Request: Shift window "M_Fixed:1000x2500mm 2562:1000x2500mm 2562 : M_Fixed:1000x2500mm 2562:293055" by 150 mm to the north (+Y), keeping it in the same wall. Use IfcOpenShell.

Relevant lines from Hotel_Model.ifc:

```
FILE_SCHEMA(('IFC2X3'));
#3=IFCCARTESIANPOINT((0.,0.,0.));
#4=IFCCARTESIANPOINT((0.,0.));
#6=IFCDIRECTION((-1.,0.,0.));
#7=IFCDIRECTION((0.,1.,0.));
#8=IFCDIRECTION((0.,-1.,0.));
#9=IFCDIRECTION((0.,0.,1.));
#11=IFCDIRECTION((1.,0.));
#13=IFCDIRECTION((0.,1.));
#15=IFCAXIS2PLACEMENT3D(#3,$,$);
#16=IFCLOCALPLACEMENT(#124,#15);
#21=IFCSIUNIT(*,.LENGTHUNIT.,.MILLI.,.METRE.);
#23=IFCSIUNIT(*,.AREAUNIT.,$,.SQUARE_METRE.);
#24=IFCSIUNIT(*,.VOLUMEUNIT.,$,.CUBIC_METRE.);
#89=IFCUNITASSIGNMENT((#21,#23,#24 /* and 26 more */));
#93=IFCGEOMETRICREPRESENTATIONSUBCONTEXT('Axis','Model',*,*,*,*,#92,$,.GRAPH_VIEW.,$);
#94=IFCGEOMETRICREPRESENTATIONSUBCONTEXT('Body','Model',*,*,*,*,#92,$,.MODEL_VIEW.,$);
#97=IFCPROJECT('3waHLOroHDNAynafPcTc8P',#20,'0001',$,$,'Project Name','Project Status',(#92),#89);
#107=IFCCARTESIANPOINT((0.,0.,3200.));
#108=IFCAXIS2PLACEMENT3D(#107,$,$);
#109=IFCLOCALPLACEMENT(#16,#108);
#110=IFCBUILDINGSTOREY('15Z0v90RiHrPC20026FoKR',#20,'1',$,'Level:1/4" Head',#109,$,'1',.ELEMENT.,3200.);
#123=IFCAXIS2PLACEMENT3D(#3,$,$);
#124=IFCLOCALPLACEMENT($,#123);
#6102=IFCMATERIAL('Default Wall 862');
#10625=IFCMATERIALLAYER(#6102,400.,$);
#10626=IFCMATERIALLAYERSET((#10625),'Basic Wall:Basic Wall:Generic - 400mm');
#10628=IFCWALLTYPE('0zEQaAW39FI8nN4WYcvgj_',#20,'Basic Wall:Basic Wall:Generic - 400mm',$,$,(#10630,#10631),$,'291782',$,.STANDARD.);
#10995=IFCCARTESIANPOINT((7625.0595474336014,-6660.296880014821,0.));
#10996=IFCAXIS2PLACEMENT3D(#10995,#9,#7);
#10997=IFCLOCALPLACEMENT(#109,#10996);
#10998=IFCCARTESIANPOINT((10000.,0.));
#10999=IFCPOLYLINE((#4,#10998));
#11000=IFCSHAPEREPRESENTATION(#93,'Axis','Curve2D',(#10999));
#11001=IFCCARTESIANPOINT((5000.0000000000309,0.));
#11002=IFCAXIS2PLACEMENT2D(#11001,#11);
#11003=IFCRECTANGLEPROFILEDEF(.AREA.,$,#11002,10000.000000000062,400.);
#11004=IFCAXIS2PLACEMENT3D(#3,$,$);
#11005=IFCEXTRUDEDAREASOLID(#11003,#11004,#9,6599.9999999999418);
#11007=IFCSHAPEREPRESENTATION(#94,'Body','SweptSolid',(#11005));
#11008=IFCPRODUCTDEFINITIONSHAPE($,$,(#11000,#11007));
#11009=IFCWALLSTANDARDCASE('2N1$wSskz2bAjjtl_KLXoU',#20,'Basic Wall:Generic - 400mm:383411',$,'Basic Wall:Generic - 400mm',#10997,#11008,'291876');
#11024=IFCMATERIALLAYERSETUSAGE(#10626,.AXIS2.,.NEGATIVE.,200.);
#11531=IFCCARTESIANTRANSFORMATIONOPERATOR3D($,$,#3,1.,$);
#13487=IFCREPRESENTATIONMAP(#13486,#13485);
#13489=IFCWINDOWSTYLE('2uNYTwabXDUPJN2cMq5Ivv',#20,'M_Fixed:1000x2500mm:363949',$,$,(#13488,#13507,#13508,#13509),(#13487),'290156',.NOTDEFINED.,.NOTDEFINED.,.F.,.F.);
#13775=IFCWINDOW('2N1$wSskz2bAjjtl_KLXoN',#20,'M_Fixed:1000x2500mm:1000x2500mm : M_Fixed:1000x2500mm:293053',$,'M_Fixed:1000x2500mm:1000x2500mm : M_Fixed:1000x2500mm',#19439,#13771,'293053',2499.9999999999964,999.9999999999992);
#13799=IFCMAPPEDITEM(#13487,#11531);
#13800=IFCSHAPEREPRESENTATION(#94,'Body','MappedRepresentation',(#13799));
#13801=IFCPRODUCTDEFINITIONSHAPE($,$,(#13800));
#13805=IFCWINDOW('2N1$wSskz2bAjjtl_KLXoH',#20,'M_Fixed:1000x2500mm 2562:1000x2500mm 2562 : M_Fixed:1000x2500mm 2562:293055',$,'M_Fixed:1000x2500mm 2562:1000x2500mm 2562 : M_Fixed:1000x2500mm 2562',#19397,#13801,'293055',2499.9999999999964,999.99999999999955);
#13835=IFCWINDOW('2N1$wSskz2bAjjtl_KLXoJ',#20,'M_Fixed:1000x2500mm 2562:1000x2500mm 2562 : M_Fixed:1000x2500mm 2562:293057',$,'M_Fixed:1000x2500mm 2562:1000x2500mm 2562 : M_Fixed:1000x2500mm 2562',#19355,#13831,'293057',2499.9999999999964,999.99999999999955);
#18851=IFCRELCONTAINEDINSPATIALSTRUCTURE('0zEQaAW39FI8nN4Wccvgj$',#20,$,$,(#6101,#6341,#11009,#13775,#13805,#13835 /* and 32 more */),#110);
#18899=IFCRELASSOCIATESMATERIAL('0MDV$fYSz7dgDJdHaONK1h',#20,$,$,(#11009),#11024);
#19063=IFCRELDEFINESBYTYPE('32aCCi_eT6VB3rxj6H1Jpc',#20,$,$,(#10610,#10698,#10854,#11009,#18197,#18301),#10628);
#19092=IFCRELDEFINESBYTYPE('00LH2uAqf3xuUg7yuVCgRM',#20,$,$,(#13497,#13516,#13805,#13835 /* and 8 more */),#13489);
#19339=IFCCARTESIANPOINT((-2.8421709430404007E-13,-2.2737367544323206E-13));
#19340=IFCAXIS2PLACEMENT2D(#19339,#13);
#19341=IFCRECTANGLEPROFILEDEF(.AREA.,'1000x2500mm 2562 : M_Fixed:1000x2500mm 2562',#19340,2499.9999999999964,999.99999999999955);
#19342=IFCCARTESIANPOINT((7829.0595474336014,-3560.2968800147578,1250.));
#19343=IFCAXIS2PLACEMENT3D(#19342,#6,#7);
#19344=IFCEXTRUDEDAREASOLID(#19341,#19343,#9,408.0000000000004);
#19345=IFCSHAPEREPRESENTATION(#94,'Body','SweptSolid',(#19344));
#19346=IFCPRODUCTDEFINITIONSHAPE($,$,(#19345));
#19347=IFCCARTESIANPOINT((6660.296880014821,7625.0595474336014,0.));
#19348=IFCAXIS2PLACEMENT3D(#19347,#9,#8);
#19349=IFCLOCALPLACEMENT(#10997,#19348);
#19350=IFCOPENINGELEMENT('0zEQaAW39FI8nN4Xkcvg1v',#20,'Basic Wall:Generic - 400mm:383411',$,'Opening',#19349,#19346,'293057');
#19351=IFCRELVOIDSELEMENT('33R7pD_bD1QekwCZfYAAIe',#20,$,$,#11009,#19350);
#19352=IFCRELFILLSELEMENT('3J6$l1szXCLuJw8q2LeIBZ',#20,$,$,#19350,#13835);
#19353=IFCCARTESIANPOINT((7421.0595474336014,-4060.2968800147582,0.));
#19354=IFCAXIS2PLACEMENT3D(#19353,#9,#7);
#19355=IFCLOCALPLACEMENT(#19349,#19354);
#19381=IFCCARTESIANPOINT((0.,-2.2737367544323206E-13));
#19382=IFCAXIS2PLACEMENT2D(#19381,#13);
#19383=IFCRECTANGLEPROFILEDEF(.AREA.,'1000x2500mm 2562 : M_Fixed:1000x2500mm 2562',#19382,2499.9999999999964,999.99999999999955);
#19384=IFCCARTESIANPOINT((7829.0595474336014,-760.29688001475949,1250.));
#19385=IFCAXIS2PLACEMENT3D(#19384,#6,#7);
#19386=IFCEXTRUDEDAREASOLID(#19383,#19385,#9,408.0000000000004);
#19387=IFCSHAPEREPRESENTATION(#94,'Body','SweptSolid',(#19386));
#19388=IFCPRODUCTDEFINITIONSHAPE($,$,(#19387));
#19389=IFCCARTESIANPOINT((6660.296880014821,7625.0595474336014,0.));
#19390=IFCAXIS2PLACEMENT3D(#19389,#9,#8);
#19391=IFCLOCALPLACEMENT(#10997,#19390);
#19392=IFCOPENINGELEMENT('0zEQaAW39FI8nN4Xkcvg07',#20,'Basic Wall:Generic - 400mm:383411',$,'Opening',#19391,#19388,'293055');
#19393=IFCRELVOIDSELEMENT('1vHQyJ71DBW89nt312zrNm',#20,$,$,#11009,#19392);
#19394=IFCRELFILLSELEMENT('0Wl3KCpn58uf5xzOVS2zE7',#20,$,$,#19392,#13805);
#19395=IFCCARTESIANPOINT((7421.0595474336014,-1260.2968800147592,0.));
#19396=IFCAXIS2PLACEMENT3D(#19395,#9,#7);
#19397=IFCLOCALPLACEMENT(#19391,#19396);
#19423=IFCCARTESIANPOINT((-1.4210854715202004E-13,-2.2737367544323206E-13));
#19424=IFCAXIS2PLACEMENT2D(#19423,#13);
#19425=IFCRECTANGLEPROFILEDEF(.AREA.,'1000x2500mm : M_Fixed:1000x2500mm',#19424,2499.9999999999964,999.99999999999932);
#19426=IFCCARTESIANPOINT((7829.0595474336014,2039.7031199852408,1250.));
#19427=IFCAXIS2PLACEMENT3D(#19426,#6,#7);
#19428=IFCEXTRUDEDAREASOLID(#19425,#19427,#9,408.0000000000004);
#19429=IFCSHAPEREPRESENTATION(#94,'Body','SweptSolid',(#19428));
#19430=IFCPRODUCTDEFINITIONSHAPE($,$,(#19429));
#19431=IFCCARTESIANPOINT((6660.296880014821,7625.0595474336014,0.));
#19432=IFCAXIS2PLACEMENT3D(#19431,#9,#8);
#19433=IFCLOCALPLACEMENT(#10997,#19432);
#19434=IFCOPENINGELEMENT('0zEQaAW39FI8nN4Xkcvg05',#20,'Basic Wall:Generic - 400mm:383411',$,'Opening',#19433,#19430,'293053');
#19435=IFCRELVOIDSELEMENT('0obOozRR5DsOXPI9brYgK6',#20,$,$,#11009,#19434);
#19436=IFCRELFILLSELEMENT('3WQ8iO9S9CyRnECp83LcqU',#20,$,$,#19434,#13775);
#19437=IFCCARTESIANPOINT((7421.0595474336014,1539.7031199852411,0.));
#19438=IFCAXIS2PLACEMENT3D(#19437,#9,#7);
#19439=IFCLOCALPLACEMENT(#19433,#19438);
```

```python
import ifcopenshell
import ifcopenshell.api.geometry
import ifcopenshell.util.placement

model = ifcopenshell.open("Hotel_Model.ifc")

window = model.by_guid("2N1$wSskz2bAjjtl_KLXoH")
opening = window.FillsVoids[0].RelatingOpeningElement
wall = opening.VoidsElements[0].RelatingBuildingElement

wall_matrix = ifcopenshell.util.placement.get_local_placement(wall.ObjectPlacement)
shift = wall_matrix[:3, 0] * 150.0
before = ifcopenshell.util.placement.get_local_placement(window.ObjectPlacement)[:3, 3].copy()

# The window is placed relative to its opening, so it follows when the opening moves.
matrix = ifcopenshell.util.placement.get_local_placement(opening.ObjectPlacement)
matrix[:3, 3] += shift
ifcopenshell.api.geometry.edit_object_placement(
    model, product=opening, matrix=matrix, is_si=False, should_transform_children=True
)

after = ifcopenshell.util.placement.get_local_placement(window.ObjectPlacement)[:3, 3]
print("window moved by", (after - before).round(3) + 0.0)

model.write("Hotel_Model_updated.ifc")
```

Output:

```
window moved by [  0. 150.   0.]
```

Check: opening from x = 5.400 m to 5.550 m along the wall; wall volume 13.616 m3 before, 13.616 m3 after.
